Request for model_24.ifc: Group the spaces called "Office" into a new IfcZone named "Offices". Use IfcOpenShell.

First a look at what the model holds.

```python
import ifcopenshell

model = ifcopenshell.open("model_24.ifc")
print(model.schema)
seen = {}
for space in model.by_type("IfcSpace"):
    seen[space.LongName] = seen.get(space.LongName, 0) + 1
for name, count in sorted(seen.items(), key=str):
    print(count, "x", name)
print("zones:", [z.Name for z in model.by_type("IfcZone")][:20])
```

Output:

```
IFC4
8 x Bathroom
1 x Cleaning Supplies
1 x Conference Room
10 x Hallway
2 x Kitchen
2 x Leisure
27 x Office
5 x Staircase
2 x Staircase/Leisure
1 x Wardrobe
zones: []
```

```python
import ifcopenshell
import ifcopenshell.api.group
import ifcopenshell.api.root

model = ifcopenshell.open("model_24.ifc")

names = {"Office"}
spaces = [s for s in model.by_type("IfcSpace") if s.LongName in names]

zone = ifcopenshell.api.root.create_entity(model, ifc_class="IfcZone", name="Offices")
ifcopenshell.api.group.assign_group(model, products=spaces, group=zone)
print(len(spaces), "spaces in", zone.Name)

model.write("model_24_rev.ifc")
```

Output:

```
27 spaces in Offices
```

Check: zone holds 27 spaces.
